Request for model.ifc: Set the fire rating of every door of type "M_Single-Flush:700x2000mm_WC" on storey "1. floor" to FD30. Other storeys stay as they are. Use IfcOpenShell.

First a look at what the model holds.

```python
import ifcopenshell
import ifcopenshell.util.element

model = ifcopenshell.open("model.ifc")
print(model.schema)
storey = next(s for s in model.by_type("IfcBuildingStorey") if s.Name == "1. floor")
doors = [e for e in ifcopenshell.util.element.get_decomposition(storey) if e.is_a("IfcDoor")]
seen = {}
for e in doors:
    element_type = ifcopenshell.util.element.get_type(e)
    key = (element_type.Name if element_type != e and element_type else None, ifcopenshell.util.element.get_pset(e, "Pset_DoorCommon", "FireRating"))
    seen[key] = seen.get(key, 0) + 1
for (name, value), count in sorted(seen.items(), key=str):
    print(count, "x", name, "|", value)
```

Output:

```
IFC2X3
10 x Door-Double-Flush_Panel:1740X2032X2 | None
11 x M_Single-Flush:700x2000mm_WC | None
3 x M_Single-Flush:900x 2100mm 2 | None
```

```python
import ifcopenshell
import ifcopenshell.api.pset
import ifcopenshell.util.element

model = ifcopenshell.open("model.ifc")

storey = next(s for s in model.by_type("IfcBuildingStorey") if s.Name == "1. floor")
doors = [e for e in ifcopenshell.util.element.get_decomposition(storey) if e.is_a("IfcDoor")]

count = 0
for e in doors:
    element_type = ifcopenshell.util.element.get_type(e)
    if element_type in (None, e) or element_type.Name != "M_Single-Flush:700x2000mm_WC":
        continue
    # add_pset returns the element's existing set when there is one.
    pset = ifcopenshell.api.pset.add_pset(model, product=e, name="Pset_DoorCommon")
    ifcopenshell.api.pset.edit_pset(model, pset=pset, properties={"FireRating": "FD30"})
    count += 1

print(count, "doors updated")

model.write("model_edited.ifc")
```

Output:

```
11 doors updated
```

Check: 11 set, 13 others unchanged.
